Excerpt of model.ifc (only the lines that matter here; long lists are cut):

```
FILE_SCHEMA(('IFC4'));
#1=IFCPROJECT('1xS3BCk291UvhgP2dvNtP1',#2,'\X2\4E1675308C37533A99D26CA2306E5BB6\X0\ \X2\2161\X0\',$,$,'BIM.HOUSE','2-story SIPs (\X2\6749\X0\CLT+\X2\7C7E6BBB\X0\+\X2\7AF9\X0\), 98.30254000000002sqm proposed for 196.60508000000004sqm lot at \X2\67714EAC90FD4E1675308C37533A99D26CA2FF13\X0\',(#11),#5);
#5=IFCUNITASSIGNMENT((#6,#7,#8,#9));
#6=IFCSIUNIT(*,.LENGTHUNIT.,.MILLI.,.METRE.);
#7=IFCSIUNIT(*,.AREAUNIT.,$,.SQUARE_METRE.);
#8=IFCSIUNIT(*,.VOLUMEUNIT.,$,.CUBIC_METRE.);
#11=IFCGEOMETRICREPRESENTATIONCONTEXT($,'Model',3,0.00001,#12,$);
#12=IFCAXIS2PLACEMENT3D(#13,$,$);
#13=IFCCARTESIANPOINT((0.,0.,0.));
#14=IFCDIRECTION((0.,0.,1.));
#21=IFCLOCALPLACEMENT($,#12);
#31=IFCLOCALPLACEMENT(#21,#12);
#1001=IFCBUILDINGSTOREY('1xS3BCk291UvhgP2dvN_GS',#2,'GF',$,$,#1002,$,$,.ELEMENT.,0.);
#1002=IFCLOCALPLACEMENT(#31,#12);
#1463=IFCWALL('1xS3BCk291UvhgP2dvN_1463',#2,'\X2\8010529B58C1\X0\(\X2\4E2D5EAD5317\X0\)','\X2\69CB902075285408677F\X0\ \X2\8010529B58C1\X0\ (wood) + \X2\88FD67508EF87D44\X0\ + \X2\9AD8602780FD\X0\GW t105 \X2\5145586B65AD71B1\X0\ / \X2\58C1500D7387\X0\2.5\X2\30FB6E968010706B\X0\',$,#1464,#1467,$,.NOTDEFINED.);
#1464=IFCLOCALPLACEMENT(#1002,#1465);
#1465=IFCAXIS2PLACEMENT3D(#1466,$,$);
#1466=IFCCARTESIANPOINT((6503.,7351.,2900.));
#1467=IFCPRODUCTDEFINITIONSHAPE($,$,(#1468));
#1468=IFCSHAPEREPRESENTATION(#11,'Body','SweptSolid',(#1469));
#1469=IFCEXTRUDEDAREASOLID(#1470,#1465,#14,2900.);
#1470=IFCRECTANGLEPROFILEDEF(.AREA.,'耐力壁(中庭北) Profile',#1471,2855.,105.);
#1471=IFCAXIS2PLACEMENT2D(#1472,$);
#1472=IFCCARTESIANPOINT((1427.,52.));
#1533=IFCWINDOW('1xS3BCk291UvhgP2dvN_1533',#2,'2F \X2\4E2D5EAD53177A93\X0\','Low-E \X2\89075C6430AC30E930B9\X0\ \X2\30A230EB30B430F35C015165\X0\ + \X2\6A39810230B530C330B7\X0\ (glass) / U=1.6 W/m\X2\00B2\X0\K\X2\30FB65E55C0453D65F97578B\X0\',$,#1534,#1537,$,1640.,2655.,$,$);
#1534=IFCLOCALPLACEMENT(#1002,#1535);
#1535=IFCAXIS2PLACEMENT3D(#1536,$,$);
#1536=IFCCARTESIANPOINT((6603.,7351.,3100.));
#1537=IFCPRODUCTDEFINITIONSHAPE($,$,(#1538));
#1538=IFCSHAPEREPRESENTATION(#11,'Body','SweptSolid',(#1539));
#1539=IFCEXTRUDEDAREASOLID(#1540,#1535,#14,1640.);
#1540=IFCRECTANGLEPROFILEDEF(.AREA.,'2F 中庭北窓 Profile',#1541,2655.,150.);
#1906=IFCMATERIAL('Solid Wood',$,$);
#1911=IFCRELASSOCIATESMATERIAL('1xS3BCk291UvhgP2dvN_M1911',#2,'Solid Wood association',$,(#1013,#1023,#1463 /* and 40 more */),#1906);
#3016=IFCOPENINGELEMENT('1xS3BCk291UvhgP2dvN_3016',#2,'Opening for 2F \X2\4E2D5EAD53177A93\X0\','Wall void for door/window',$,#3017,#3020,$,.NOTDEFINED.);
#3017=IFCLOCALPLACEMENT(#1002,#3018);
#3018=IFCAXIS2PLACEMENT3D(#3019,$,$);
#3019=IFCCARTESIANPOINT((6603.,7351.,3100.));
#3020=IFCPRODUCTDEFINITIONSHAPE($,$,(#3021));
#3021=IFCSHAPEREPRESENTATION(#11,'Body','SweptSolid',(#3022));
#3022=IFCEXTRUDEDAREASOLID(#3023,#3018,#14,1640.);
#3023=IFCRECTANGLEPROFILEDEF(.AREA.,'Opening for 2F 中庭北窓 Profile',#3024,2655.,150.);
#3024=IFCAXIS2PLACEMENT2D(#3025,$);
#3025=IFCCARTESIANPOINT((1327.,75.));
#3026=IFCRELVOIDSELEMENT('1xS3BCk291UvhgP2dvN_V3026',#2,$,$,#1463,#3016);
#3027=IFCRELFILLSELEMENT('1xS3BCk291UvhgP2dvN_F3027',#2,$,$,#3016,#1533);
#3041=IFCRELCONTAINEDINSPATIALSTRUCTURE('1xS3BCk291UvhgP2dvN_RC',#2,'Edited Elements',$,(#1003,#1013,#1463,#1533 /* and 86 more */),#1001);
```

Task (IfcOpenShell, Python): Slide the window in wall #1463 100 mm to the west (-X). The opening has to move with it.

```python
import ifcopenshell
import ifcopenshell.api.geometry
import ifcopenshell.util.placement
import ifcopenshell.util.unit

model = ifcopenshell.open("model.ifc")
unit_scale = ifcopenshell.util.unit.calculate_unit_scale(model)

window = model.by_guid("1xS3BCk291UvhgP2dvN_1533")
opening = window.FillsVoids[0].RelatingOpeningElement
wall = opening.VoidsElements[0].RelatingBuildingElement

wall_matrix = ifcopenshell.util.placement.get_local_placement(wall.ObjectPlacement)
shift = wall_matrix[:3, 0] * -0.1 / unit_scale
before = ifcopenshell.util.placement.get_local_placement(window.ObjectPlacement)[:3, 3].copy()

# The window is not placed relative to its opening, so move both.
for product in (opening, window):
    matrix = ifcopenshell.util.placement.get_local_placement(product.ObjectPlacement)
    matrix[:3, 3] += shift
    ifcopenshell.api.geometry.edit_object_placement(model, product=product, matrix=matrix, is_si=False)

after = ifcopenshell.util.placement.get_local_placement(window.ObjectPlacement)[:3, 3]
print("window moved by", (after - before).round(3) + 0.0)

model.write("model_rev.ifc")
```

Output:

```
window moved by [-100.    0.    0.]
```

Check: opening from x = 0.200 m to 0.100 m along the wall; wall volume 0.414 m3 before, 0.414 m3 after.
